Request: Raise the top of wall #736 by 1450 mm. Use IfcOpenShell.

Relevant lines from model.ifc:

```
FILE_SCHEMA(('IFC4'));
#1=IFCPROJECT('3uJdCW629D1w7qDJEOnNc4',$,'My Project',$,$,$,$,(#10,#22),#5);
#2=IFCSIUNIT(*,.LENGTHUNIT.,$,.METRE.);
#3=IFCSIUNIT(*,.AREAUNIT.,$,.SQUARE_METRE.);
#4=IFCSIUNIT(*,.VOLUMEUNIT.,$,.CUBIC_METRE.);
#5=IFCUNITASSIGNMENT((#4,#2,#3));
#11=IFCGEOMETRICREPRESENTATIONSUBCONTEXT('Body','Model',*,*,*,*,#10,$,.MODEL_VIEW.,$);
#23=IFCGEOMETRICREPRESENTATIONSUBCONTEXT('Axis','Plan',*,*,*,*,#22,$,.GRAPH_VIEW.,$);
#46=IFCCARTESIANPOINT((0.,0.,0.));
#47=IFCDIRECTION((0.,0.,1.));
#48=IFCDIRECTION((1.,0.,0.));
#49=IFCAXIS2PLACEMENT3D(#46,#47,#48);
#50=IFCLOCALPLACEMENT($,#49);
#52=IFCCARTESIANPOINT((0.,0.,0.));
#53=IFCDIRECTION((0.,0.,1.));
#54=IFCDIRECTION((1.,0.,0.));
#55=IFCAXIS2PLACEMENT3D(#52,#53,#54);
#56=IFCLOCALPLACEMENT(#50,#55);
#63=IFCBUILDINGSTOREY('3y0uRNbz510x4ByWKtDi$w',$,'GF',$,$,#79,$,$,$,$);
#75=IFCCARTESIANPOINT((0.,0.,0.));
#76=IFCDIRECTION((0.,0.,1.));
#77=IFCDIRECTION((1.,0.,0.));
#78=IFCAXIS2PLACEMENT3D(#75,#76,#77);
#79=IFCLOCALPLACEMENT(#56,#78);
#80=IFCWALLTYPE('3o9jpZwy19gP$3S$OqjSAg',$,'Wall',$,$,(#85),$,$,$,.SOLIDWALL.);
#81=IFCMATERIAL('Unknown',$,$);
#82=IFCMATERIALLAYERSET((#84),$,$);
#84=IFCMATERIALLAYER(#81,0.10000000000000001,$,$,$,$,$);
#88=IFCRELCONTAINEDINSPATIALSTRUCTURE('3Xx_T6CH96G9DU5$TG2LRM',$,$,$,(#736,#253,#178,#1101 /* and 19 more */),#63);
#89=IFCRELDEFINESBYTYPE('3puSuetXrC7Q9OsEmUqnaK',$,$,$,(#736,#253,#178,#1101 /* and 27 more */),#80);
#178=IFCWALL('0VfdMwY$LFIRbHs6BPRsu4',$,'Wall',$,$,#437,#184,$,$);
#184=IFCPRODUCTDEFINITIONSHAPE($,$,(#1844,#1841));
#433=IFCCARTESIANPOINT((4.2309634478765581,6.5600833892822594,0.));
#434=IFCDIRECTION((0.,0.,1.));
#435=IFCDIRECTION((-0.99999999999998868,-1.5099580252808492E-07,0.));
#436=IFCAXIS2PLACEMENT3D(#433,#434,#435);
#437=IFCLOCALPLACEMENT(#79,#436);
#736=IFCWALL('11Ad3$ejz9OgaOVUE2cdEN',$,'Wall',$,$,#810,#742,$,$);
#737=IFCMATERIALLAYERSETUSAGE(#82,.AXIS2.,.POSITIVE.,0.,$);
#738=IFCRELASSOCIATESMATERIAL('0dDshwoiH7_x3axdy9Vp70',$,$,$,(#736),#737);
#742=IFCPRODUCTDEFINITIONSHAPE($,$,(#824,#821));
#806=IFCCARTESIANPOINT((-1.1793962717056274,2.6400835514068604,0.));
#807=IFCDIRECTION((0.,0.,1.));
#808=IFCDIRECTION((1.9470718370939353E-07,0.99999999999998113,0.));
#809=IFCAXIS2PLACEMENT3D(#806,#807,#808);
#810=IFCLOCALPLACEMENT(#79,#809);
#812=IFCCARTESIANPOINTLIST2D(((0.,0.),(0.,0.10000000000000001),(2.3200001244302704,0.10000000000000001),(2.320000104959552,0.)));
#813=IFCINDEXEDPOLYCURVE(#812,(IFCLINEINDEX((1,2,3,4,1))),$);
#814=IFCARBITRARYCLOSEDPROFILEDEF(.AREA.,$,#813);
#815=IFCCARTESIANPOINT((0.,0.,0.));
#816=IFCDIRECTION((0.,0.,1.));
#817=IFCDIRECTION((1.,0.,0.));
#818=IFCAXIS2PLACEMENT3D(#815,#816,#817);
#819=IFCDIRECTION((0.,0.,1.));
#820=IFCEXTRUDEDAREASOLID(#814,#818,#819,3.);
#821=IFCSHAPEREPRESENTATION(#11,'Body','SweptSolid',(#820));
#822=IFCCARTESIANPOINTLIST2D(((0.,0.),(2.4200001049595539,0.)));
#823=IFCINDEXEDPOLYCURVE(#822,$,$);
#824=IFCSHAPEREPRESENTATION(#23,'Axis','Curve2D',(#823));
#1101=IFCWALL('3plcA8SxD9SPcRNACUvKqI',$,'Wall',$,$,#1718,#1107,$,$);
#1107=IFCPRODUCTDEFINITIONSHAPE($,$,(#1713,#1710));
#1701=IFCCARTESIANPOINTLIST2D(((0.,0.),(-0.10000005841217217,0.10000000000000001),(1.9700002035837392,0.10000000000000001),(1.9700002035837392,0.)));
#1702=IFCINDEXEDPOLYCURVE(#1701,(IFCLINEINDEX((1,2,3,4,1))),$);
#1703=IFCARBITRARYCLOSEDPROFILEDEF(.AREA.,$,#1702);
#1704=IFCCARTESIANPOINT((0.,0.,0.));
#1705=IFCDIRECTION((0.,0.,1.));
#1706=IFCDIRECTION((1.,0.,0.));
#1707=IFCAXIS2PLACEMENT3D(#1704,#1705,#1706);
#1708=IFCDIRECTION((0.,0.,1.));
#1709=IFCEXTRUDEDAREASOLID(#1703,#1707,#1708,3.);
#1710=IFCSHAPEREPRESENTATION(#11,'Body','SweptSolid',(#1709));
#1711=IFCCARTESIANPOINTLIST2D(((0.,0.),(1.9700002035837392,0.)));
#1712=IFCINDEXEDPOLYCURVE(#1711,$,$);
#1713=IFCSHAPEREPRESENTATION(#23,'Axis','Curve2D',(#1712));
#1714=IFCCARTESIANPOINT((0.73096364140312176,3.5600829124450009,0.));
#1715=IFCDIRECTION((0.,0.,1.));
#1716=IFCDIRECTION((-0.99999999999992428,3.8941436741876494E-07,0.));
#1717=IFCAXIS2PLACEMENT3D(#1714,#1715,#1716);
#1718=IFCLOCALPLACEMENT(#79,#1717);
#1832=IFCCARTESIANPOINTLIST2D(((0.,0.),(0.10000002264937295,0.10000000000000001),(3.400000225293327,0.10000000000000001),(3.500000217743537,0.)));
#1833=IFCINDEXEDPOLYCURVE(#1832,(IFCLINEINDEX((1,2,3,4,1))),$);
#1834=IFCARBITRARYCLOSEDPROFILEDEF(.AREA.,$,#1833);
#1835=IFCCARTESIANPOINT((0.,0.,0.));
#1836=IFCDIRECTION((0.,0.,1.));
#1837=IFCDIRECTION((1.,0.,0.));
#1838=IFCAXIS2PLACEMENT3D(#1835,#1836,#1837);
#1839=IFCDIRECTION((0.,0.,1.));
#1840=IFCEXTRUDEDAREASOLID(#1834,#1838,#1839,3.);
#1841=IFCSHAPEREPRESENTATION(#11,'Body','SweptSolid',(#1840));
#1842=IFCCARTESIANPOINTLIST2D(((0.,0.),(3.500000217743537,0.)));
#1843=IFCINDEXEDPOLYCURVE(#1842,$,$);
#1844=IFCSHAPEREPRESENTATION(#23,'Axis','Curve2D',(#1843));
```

```python
import ifcopenshell
import ifcopenshell.geom
import ifcopenshell.util.representation
import ifcopenshell.util.shape
import ifcopenshell.util.unit

model = ifcopenshell.open("model.ifc")
unit_scale = ifcopenshell.util.unit.calculate_unit_scale(model)
settings = ifcopenshell.geom.settings()


def volume(element):
    """Net volume in cubic metres, openings subtracted."""
    shape = ifcopenshell.geom.create_shape(settings, element)
    return ifcopenshell.util.shape.get_volume(shape.geometry)


wall = model.by_guid("11Ad3$ejz9OgaOVUE2cdEN")
before = volume(wall)

body = ifcopenshell.util.representation.get_representation(wall, "Model", "Body")
solid = body.Items[0]
old_height = solid.Depth
solid.Depth += 1.45 / unit_scale
after = volume(wall)

print(f"height {old_height:g} -> {solid.Depth:g}, volume {before:.3f} -> {after:.3f} m3")

model.write("model_updated.ifc")
```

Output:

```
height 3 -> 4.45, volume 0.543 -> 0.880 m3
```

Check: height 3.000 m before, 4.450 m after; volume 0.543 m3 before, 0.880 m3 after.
